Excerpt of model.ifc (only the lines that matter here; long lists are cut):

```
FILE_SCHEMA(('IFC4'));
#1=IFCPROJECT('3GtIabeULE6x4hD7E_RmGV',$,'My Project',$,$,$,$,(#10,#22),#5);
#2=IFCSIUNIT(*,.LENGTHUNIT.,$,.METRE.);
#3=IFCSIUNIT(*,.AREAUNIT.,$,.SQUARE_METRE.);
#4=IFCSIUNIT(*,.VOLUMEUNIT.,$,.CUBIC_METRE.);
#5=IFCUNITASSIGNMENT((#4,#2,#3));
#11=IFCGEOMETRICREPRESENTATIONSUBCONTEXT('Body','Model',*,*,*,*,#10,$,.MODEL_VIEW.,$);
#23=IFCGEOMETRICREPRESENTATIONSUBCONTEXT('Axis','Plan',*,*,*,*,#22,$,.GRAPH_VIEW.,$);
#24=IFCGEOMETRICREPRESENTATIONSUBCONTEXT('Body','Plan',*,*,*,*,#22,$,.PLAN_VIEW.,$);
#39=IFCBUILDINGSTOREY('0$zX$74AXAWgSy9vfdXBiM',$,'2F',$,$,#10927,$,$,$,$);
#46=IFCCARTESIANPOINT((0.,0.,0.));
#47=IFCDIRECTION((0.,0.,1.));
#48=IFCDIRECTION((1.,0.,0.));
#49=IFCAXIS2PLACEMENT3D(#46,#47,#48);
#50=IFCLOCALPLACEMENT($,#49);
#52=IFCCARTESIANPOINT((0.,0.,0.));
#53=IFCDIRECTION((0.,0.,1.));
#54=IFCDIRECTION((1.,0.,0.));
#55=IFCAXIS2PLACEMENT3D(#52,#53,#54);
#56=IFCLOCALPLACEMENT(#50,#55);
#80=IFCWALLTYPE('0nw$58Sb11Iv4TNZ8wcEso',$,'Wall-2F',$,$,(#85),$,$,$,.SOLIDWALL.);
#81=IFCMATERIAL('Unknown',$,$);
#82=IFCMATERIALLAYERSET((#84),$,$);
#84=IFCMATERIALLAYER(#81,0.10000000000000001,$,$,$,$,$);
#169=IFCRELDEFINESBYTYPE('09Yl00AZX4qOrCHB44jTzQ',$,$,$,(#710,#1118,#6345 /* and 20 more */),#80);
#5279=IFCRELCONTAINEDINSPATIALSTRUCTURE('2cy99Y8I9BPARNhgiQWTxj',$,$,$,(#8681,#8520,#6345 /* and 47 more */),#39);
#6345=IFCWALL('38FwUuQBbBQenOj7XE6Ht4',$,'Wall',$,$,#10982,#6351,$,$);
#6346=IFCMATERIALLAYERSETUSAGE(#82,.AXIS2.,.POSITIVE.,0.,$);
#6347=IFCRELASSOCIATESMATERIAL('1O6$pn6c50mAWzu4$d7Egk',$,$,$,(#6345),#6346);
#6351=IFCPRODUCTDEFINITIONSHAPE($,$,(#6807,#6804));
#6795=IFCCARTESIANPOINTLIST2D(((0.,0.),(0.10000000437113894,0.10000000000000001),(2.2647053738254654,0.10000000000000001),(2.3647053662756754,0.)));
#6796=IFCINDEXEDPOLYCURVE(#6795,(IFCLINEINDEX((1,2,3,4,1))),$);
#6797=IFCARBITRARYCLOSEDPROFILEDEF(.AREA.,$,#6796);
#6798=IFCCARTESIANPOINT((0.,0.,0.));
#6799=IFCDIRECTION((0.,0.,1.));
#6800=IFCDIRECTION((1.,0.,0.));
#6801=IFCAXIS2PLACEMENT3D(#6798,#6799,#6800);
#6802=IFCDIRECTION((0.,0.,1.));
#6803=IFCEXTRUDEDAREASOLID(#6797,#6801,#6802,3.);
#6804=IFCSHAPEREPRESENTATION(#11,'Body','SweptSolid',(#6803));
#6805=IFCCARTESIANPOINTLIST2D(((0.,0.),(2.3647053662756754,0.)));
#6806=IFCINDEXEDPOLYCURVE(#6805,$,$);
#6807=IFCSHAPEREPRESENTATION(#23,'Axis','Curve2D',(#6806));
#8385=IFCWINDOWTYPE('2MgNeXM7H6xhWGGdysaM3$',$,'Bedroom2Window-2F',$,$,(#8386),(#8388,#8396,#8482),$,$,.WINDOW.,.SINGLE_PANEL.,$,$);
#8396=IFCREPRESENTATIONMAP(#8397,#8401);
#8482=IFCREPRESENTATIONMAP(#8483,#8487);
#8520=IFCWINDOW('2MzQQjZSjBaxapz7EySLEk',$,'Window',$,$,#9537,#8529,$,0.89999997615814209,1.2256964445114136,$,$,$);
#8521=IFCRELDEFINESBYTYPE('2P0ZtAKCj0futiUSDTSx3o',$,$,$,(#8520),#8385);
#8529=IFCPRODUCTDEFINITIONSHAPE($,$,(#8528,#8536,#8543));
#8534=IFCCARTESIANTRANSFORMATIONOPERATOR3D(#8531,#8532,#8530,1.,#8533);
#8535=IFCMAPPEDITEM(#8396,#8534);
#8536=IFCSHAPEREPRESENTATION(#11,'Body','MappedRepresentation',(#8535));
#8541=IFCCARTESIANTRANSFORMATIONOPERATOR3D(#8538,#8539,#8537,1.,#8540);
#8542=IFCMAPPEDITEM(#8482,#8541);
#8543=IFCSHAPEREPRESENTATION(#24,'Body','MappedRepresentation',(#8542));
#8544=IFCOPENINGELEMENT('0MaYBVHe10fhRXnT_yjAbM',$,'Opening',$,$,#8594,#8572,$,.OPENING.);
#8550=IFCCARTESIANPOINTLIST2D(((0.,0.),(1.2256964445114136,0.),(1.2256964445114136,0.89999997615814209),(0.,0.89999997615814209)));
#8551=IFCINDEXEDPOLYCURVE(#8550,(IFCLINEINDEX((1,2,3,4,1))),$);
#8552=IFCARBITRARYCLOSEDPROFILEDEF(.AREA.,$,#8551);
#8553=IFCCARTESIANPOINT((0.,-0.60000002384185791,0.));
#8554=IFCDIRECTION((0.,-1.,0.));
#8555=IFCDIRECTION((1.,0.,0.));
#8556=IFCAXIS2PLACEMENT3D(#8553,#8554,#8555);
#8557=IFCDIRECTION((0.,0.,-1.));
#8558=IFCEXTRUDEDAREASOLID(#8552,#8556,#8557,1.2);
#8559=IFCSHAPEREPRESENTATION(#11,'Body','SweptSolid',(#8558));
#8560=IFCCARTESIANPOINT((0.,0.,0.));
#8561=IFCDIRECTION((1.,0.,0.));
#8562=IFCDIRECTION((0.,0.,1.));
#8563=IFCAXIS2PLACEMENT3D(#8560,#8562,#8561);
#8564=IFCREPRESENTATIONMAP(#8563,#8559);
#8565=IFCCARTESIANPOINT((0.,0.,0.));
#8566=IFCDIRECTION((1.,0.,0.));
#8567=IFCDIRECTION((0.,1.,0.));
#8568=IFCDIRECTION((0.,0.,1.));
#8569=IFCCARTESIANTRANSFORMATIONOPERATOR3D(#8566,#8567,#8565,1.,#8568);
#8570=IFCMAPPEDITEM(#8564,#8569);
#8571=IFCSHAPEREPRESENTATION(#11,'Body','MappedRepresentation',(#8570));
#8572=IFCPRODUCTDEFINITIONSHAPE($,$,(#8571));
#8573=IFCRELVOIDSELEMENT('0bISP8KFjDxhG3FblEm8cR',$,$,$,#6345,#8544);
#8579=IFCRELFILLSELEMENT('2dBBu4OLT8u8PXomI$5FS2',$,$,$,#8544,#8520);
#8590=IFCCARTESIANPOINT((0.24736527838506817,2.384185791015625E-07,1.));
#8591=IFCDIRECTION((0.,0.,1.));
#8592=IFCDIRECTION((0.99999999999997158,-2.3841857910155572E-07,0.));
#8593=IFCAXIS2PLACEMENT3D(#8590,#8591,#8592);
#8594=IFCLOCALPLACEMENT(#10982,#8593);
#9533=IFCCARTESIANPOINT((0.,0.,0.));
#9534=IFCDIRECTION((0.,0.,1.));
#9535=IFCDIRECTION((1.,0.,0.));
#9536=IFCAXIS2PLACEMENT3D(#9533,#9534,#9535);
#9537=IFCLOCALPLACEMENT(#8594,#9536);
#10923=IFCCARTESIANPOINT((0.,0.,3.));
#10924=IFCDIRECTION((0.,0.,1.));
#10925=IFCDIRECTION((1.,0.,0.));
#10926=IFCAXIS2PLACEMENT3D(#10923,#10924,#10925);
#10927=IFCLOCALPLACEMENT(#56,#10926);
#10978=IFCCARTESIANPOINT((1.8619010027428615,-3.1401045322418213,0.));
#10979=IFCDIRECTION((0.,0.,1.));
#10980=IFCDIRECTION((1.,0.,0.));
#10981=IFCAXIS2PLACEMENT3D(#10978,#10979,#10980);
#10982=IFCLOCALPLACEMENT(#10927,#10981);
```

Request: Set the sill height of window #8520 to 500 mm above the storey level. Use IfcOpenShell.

```python
import numpy as np
import ifcopenshell
import ifcopenshell.api.geometry
import ifcopenshell.geom
import ifcopenshell.util.element
import ifcopenshell.util.placement
import ifcopenshell.util.shape
import ifcopenshell.util.unit

model = ifcopenshell.open("model.ifc")
unit_scale = ifcopenshell.util.unit.calculate_unit_scale(model)

window = model.by_guid("2MzQQjZSjBaxapz7EySLEk")
opening = window.FillsVoids[0].RelatingOpeningElement
storey = ifcopenshell.util.element.get_container(window, ifc_class="IfcBuildingStorey")
level = ifcopenshell.util.placement.get_local_placement(storey.ObjectPlacement)[2, 3]

# The opening's origin need not be at the sill, so measure its lowest point.
shape = ifcopenshell.geom.create_shape(ifcopenshell.geom.settings(), opening)
bottom = ifcopenshell.util.shape.get_shape_bottom_elevation(shape, shape.geometry) / unit_scale
dz = level + 0.5 / unit_scale - bottom

shift = np.array([0.0, 0.0, dz])
# The window is placed relative to its opening, so it follows when the opening moves.
matrix = ifcopenshell.util.placement.get_local_placement(opening.ObjectPlacement)
matrix[:3, 3] += shift
ifcopenshell.api.geometry.edit_object_placement(
    model, product=opening, matrix=matrix, is_si=False, should_transform_children=True
)

print(f"moved by {dz * unit_scale:+.3f} m")

model.write("model_rev.ifc")
```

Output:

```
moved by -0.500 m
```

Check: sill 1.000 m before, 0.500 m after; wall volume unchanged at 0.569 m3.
